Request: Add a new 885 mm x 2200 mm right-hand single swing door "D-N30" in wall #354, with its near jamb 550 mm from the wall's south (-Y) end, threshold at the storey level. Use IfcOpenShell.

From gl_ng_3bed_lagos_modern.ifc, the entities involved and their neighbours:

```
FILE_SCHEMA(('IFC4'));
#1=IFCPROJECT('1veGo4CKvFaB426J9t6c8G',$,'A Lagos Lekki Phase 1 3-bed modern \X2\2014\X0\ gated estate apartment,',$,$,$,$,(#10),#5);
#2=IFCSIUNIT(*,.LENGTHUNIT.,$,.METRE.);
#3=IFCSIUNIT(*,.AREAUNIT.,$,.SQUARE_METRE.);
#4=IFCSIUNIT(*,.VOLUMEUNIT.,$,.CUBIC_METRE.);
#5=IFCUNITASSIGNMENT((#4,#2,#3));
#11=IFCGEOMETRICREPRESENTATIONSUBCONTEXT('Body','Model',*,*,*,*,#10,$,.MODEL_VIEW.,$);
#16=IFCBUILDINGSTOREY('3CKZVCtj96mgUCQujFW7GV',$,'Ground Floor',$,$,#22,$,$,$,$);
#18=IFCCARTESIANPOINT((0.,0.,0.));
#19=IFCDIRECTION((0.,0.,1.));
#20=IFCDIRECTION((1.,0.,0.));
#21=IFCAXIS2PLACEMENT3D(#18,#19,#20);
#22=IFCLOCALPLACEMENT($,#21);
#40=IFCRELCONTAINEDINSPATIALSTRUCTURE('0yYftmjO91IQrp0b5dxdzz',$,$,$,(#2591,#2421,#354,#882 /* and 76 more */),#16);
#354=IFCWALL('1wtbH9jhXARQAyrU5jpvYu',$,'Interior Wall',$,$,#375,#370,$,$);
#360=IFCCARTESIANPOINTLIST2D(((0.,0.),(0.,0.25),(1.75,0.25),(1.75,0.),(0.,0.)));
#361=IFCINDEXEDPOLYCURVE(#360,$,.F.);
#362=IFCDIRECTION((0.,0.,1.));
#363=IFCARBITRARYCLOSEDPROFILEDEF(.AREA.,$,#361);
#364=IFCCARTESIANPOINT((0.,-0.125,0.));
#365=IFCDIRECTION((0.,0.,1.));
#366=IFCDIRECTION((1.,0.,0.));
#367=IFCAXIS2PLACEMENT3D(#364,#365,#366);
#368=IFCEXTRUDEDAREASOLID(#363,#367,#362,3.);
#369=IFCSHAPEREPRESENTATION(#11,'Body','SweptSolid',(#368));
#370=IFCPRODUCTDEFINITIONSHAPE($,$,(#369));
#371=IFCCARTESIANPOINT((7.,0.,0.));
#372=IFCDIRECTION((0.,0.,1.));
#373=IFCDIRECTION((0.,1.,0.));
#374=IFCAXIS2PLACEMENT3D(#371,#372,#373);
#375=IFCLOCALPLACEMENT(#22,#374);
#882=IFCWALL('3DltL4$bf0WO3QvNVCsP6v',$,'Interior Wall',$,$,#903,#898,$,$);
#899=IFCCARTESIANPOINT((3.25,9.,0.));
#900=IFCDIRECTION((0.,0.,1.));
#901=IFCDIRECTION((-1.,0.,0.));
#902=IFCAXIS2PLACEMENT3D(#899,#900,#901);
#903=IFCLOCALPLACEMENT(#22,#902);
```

```python
import numpy as np
import ifcopenshell
import ifcopenshell.api.feature
import ifcopenshell.api.geometry
import ifcopenshell.api.root
import ifcopenshell.api.spatial
import ifcopenshell.geom
import ifcopenshell.util.element
import ifcopenshell.util.placement
import ifcopenshell.util.representation
import ifcopenshell.util.shape
import ifcopenshell.util.unit

model = ifcopenshell.open("gl_ng_3bed_lagos_modern.ifc")
unit_scale = ifcopenshell.util.unit.calculate_unit_scale(model)
settings = ifcopenshell.geom.settings()


def volume(element):
    """Net volume in cubic metres, openings subtracted."""
    shape = ifcopenshell.geom.create_shape(settings, element)
    return ifcopenshell.util.shape.get_volume(shape.geometry)


wall = model.by_guid("1wtbH9jhXARQAyrU5jpvYu")
storey = ifcopenshell.util.element.get_container(wall, ifc_class="IfcBuildingStorey")
context = ifcopenshell.util.representation.get_context(model, "Model", "Body", "MODEL_VIEW")
before = volume(wall)

width, height, from_end, sill = 0.885, 2.2, 0.55, 0.0  # metres

# The wall runs along its own X axis, and the end named is its -X end.
wall_shape = ifcopenshell.geom.create_shape(settings, wall)
x, y, z = ifcopenshell.util.shape.get_vertices(wall_shape.geometry).T
start = x.min() + from_end
face, thickness = float(y.min()), float(y.max() - y.min())
wall_matrix = ifcopenshell.util.placement.get_local_placement(wall.ObjectPlacement)
level = ifcopenshell.util.placement.get_local_placement(storey.ObjectPlacement)[2, 3]


def in_wall(x, y):
    """Placement at x, y metres in the wall's axes, at sill height."""
    matrix = wall_matrix.copy()
    matrix[:, 3] = wall_matrix @ np.array([x / unit_scale, y / unit_scale, 0.0, 1.0])
    matrix[2, 3] = level + sill / unit_scale
    return matrix


# Opening: a box that overshoots both wall faces by 50 mm.
opening = ifcopenshell.api.root.create_entity(model, ifc_class="IfcOpeningElement", predefined_type="OPENING")
box = ifcopenshell.api.geometry.add_wall_representation(
    model, context=context, length=width, height=height, thickness=thickness + 0.1
)
ifcopenshell.api.geometry.assign_representation(model, product=opening, representation=box)
ifcopenshell.api.geometry.edit_object_placement(model, product=opening, matrix=in_wall(start, face - 0.05), is_si=False)
ifcopenshell.api.feature.add_feature(model, feature=opening, element=wall)

door = ifcopenshell.api.root.create_entity(model, ifc_class="IfcDoor", name="D-N30", predefined_type="DOOR")
door.OverallWidth, door.OverallHeight = width / unit_scale, height / unit_scale
door.OperationType = "SINGLE_SWING_RIGHT"
body = ifcopenshell.api.geometry.add_door_representation(
    model,
    context=context,
    overall_width=door.OverallWidth,
    overall_height=door.OverallHeight,
    operation_type="SINGLE_SWING_RIGHT",
    lining_properties={"LiningDepth": thickness / unit_scale, "ThresholdDepth": thickness / unit_scale},
)
ifcopenshell.api.geometry.assign_representation(model, product=door, representation=body)
ifcopenshell.api.spatial.assign_container(model, products=[door], relating_structure=storey)
ifcopenshell.api.feature.add_filling(model, opening=opening, element=door)

# The lining spans the wall, so the door starts at the wall face.
ifcopenshell.api.geometry.edit_object_placement(model, product=door, matrix=in_wall(start, face), is_si=False)

after = volume(wall)

print(f"wall volume {before:.3f} -> {after:.3f} m3")

model.write("gl_ng_3bed_lagos_modern_v2.ifc")
```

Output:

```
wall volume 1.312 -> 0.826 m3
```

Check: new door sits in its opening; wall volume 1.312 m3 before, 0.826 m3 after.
